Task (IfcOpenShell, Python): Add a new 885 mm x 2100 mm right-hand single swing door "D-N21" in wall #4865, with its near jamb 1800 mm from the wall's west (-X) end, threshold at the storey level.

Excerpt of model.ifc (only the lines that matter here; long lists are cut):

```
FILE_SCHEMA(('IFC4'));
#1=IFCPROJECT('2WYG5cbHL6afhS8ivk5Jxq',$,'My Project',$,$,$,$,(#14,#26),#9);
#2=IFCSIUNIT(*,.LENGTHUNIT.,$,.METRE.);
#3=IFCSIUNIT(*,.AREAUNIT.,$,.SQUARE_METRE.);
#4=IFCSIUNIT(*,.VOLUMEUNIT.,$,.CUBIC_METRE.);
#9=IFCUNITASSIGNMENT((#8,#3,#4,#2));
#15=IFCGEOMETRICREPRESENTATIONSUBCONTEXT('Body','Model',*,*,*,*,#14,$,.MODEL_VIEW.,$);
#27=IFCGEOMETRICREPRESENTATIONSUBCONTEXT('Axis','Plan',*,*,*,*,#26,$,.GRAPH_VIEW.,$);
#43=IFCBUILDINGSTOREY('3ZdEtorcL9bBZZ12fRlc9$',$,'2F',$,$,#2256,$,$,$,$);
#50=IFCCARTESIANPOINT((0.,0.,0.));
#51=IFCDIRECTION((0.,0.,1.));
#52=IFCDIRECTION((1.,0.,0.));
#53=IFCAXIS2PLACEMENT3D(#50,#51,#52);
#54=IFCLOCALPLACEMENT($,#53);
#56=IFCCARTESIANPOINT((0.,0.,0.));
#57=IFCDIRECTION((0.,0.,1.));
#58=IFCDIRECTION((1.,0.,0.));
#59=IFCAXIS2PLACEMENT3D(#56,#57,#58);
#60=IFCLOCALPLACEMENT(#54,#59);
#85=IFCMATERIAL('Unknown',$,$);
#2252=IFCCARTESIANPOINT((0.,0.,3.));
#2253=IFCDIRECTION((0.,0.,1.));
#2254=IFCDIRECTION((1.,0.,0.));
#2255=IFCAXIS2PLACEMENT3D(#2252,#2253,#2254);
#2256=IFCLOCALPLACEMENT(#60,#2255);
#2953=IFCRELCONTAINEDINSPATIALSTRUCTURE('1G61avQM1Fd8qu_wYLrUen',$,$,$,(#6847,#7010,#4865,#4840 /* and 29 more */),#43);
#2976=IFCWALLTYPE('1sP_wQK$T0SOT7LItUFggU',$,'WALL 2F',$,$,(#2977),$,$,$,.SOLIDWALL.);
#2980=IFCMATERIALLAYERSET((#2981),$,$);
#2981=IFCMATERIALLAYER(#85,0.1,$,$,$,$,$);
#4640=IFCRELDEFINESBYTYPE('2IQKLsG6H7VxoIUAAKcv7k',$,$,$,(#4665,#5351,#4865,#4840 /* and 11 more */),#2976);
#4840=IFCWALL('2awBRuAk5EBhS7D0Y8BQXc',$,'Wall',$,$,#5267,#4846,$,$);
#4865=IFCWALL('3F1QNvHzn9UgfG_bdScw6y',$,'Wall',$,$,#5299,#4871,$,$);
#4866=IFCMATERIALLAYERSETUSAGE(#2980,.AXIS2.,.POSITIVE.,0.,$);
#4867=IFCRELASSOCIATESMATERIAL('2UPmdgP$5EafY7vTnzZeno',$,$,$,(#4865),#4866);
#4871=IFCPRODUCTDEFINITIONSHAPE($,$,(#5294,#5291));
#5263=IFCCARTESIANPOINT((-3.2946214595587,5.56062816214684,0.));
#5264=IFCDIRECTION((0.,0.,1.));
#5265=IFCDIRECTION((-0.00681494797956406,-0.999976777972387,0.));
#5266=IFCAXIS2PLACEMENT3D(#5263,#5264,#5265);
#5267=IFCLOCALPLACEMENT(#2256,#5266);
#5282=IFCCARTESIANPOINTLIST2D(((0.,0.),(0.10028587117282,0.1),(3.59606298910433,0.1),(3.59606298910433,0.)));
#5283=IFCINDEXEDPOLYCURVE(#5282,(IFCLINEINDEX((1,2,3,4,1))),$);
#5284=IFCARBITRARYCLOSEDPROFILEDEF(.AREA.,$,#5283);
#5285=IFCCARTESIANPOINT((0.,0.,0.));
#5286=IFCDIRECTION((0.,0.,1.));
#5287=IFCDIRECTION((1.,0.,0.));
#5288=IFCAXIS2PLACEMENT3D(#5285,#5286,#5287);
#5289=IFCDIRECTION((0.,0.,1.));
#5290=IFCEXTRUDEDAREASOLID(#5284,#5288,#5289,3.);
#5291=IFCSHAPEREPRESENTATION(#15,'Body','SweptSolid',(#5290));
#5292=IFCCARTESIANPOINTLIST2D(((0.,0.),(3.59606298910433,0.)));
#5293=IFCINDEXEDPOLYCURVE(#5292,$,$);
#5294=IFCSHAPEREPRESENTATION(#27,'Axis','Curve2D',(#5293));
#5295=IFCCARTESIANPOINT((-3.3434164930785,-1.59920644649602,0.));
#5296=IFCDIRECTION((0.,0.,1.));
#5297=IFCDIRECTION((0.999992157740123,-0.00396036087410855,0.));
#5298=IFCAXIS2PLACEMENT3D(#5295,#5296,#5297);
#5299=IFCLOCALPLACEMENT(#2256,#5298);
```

```python
import numpy as np
import ifcopenshell
import ifcopenshell.api.feature
import ifcopenshell.api.geometry
import ifcopenshell.api.root
import ifcopenshell.api.spatial
import ifcopenshell.geom
import ifcopenshell.util.element
import ifcopenshell.util.placement
import ifcopenshell.util.representation
import ifcopenshell.util.shape
import ifcopenshell.util.unit

model = ifcopenshell.open("model.ifc")
unit_scale = ifcopenshell.util.unit.calculate_unit_scale(model)
settings = ifcopenshell.geom.settings()


def volume(element):
    """Net volume in cubic metres, openings subtracted."""
    shape = ifcopenshell.geom.create_shape(settings, element)
    return ifcopenshell.util.shape.get_volume(shape.geometry)


wall = model.by_id(4865)
storey = ifcopenshell.util.element.get_container(wall, ifc_class="IfcBuildingStorey")
context = ifcopenshell.util.representation.get_context(model, "Model", "Body", "MODEL_VIEW")
before = volume(wall)

width, height, from_end, sill = 0.885, 2.1, 1.8, 0.0  # metres

# The wall runs along its own X axis, and the end named is its -X end.
wall_shape = ifcopenshell.geom.create_shape(settings, wall)
x, y, z = ifcopenshell.util.shape.get_vertices(wall_shape.geometry).T
start = x.min() + from_end
face, thickness = float(y.min()), float(y.max() - y.min())
wall_matrix = ifcopenshell.util.placement.get_local_placement(wall.ObjectPlacement)
level = ifcopenshell.util.placement.get_local_placement(storey.ObjectPlacement)[2, 3]


def in_wall(x, y):
    """Placement at x, y metres in the wall's axes, at sill height."""
    matrix = wall_matrix.copy()
    matrix[:, 3] = wall_matrix @ np.array([x / unit_scale, y / unit_scale, 0.0, 1.0])
    matrix[2, 3] = level + sill / unit_scale
    return matrix


# Opening: a box that overshoots both wall faces by 50 mm.
opening = ifcopenshell.api.root.create_entity(model, ifc_class="IfcOpeningElement", predefined_type="OPENING")
box = ifcopenshell.api.geometry.add_wall_representation(
    model, context=context, length=width, height=height, thickness=thickness + 0.1
)
ifcopenshell.api.geometry.assign_representation(model, product=opening, representation=box)
ifcopenshell.api.geometry.edit_object_placement(model, product=opening, matrix=in_wall(start, face - 0.05), is_si=False)
ifcopenshell.api.feature.add_feature(model, feature=opening, element=wall)

door = ifcopenshell.api.root.create_entity(model, ifc_class="IfcDoor", name="D-N21", predefined_type="DOOR")
door.OverallWidth, door.OverallHeight = width / unit_scale, height / unit_scale
door.OperationType = "SINGLE_SWING_RIGHT"
body = ifcopenshell.api.geometry.add_door_representation(
    model,
    context=context,
    overall_width=door.OverallWidth,
    overall_height=door.OverallHeight,
    operation_type="SINGLE_SWING_RIGHT",
    lining_properties={"LiningDepth": thickness / unit_scale, "ThresholdDepth": thickness / unit_scale},
)
ifcopenshell.api.geometry.assign_representation(model, product=door, representation=body)
ifcopenshell.api.spatial.assign_container(model, products=[door], relating_structure=storey)
ifcopenshell.api.feature.add_filling(model, opening=opening, element=door)

# The lining spans the wall, so the door starts at the wall face.
ifcopenshell.api.geometry.edit_object_placement(model, product=door, matrix=in_wall(start, face), is_si=False)

after = volume(wall)

print(f"wall volume {before:.3f} -> {after:.3f} m3")

model.write("model_edited.ifc")
```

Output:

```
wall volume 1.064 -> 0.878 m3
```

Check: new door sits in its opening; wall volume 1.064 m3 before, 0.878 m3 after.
